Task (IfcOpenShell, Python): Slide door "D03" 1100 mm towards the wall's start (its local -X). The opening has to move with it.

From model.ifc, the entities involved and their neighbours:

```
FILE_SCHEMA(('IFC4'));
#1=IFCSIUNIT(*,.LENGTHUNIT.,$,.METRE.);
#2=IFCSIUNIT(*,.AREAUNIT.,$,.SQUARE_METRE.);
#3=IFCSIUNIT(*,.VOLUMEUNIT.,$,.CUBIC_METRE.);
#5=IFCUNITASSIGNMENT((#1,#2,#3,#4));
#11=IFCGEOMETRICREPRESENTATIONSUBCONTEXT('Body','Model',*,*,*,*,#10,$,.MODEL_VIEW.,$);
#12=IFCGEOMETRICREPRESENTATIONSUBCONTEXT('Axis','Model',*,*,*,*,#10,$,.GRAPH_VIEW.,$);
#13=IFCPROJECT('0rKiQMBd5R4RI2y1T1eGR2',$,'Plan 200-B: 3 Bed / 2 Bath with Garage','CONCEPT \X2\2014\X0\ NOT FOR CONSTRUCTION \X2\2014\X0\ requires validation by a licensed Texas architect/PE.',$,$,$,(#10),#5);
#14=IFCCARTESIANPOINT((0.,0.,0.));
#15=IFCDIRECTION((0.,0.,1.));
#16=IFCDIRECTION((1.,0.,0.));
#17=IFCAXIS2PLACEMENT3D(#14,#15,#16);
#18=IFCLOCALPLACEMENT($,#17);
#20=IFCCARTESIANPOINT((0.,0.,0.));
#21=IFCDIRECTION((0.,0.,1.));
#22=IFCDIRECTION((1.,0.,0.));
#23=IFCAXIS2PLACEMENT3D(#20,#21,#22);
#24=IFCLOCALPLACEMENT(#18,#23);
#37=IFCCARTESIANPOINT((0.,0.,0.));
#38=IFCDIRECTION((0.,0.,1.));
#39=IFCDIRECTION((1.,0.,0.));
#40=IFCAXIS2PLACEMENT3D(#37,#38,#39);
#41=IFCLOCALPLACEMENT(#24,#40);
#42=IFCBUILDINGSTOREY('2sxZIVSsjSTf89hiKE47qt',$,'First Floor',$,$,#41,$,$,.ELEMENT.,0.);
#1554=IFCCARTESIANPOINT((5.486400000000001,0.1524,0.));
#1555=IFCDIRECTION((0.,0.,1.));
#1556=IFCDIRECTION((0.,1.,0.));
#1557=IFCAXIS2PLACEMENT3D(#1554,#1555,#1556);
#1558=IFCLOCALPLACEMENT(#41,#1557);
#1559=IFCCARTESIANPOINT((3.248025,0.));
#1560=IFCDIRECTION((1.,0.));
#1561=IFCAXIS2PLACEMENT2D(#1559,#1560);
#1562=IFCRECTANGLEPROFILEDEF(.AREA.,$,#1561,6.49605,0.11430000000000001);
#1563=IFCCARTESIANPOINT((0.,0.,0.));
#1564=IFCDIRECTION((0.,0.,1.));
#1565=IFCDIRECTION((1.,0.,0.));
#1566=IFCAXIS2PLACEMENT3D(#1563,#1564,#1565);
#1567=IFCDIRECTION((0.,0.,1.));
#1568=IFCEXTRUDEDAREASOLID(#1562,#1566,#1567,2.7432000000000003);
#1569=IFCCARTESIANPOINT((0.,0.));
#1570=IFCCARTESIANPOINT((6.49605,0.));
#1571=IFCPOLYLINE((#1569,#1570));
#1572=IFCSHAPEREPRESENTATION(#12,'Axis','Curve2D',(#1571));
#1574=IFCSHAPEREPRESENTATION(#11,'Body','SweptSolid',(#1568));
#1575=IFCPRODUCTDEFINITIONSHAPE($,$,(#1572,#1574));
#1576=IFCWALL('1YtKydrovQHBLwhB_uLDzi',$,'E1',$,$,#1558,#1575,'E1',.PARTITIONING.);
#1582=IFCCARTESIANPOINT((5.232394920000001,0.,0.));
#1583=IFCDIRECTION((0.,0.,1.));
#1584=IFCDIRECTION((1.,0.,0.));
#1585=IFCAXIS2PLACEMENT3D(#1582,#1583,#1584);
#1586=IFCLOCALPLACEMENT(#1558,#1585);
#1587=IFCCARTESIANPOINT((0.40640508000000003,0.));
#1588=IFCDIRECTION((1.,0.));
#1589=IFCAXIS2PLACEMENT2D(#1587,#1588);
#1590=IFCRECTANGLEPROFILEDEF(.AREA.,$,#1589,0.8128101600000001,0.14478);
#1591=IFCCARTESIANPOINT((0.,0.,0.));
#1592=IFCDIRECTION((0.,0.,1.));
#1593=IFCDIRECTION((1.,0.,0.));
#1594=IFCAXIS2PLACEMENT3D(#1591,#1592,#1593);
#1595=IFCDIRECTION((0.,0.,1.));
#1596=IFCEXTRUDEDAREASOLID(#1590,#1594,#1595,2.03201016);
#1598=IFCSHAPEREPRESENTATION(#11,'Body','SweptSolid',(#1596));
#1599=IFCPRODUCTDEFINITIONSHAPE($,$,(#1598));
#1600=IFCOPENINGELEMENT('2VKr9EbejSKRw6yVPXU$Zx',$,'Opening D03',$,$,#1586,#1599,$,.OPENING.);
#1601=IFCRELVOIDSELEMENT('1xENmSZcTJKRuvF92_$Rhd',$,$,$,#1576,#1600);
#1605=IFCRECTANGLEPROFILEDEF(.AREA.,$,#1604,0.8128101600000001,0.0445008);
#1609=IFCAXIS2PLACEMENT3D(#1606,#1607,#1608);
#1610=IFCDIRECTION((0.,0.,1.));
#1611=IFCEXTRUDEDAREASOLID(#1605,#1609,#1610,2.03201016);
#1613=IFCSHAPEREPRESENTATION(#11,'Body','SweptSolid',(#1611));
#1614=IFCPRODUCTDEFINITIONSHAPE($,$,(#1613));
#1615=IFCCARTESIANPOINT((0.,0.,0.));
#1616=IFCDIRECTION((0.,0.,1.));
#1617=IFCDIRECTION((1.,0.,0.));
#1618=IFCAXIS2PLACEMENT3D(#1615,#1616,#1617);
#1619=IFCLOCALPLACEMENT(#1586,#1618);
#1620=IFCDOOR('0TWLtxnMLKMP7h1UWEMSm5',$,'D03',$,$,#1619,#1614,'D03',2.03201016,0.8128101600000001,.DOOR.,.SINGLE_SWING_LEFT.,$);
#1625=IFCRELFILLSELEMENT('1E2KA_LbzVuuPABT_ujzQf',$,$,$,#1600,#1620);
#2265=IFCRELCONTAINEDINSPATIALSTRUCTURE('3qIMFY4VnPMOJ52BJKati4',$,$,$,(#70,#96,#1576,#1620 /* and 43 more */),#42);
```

```python
import ifcopenshell
import ifcopenshell.api.geometry
import ifcopenshell.util.placement
import ifcopenshell.util.unit

model = ifcopenshell.open("model.ifc")
unit_scale = ifcopenshell.util.unit.calculate_unit_scale(model)

door = model.by_id(1620)
opening = door.FillsVoids[0].RelatingOpeningElement
wall = opening.VoidsElements[0].RelatingBuildingElement

wall_matrix = ifcopenshell.util.placement.get_local_placement(wall.ObjectPlacement)
shift = wall_matrix[:3, 0] * -1.1 / unit_scale
before = ifcopenshell.util.placement.get_local_placement(door.ObjectPlacement)[:3, 3].copy()

# The door is placed relative to its opening, so it follows when the opening moves.
matrix = ifcopenshell.util.placement.get_local_placement(opening.ObjectPlacement)
matrix[:3, 3] += shift
ifcopenshell.api.geometry.edit_object_placement(
    model, product=opening, matrix=matrix, is_si=False, should_transform_children=True
)

after = ifcopenshell.util.placement.get_local_placement(door.ObjectPlacement)[:3, 3]
print("door moved by", (after - before).round(3) + 0.0)

model.write("model_v2.ifc")
```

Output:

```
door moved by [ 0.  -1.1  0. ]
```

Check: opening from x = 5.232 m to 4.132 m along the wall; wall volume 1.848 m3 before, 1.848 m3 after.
